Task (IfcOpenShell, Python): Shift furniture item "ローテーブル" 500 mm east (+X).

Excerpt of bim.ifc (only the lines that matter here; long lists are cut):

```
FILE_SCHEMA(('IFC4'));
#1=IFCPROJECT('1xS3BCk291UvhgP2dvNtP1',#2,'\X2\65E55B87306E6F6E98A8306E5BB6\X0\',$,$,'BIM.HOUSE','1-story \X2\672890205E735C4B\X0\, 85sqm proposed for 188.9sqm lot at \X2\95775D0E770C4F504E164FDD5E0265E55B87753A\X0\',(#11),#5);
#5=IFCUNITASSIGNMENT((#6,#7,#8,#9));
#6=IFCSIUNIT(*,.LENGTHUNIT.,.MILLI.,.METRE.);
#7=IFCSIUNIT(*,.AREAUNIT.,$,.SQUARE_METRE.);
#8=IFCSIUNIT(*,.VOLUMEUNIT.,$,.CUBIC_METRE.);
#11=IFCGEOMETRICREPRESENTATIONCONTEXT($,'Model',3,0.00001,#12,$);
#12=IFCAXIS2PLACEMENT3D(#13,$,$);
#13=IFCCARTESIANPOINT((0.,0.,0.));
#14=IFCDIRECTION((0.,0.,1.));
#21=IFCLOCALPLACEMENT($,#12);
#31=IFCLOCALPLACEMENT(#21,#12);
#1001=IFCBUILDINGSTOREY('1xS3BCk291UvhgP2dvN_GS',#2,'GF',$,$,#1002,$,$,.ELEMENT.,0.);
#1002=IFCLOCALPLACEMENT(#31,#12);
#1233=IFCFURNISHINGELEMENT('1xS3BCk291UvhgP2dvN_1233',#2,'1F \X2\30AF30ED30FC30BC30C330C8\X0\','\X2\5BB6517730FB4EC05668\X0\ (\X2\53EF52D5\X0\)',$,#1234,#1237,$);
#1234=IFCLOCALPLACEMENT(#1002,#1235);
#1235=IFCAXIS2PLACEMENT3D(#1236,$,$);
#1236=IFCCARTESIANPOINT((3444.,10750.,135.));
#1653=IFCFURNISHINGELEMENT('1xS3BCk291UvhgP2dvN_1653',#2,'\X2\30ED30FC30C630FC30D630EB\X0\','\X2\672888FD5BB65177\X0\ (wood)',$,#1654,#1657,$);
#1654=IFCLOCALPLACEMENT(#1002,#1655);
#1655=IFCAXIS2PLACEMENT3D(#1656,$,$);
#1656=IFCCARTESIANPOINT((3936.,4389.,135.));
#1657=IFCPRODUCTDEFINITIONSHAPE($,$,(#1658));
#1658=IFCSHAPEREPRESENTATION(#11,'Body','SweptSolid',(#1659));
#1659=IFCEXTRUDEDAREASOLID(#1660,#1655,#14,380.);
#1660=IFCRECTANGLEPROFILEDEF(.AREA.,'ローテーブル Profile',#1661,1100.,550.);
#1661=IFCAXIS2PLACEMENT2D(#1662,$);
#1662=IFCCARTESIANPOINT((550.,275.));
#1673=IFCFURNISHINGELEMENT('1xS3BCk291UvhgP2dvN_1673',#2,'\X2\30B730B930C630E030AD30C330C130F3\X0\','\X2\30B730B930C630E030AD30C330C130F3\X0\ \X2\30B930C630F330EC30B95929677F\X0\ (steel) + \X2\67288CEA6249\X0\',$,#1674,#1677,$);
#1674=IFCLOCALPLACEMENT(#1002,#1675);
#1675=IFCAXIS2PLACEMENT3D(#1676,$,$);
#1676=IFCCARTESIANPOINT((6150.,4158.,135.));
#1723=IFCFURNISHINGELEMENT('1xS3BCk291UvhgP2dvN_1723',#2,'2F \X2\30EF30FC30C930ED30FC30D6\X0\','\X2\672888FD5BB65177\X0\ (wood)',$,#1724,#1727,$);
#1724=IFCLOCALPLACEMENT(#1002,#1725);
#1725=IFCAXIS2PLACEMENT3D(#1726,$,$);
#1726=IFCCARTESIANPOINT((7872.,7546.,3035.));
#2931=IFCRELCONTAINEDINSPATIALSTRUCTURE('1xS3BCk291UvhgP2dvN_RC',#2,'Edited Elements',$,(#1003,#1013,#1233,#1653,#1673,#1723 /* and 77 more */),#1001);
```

```python
import ifcopenshell
import ifcopenshell.api.geometry
import ifcopenshell.util.placement
import ifcopenshell.util.unit

model = ifcopenshell.open("bim.ifc")
unit_scale = ifcopenshell.util.unit.calculate_unit_scale(model)

item = model.by_id(1653)
matrix = ifcopenshell.util.placement.get_local_placement(item.ObjectPlacement)
matrix[0, 3] += 0.5 / unit_scale
ifcopenshell.api.geometry.edit_object_placement(model, product=item, matrix=matrix, is_si=False)

print(ifcopenshell.util.placement.get_local_placement(item.ObjectPlacement).round(3) + 0.0)

model.write("bim_edited.ifc")
```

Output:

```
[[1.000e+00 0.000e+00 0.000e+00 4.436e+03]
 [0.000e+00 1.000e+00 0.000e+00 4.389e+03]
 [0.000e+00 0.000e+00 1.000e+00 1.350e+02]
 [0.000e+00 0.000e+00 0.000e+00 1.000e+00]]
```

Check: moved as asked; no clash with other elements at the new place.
